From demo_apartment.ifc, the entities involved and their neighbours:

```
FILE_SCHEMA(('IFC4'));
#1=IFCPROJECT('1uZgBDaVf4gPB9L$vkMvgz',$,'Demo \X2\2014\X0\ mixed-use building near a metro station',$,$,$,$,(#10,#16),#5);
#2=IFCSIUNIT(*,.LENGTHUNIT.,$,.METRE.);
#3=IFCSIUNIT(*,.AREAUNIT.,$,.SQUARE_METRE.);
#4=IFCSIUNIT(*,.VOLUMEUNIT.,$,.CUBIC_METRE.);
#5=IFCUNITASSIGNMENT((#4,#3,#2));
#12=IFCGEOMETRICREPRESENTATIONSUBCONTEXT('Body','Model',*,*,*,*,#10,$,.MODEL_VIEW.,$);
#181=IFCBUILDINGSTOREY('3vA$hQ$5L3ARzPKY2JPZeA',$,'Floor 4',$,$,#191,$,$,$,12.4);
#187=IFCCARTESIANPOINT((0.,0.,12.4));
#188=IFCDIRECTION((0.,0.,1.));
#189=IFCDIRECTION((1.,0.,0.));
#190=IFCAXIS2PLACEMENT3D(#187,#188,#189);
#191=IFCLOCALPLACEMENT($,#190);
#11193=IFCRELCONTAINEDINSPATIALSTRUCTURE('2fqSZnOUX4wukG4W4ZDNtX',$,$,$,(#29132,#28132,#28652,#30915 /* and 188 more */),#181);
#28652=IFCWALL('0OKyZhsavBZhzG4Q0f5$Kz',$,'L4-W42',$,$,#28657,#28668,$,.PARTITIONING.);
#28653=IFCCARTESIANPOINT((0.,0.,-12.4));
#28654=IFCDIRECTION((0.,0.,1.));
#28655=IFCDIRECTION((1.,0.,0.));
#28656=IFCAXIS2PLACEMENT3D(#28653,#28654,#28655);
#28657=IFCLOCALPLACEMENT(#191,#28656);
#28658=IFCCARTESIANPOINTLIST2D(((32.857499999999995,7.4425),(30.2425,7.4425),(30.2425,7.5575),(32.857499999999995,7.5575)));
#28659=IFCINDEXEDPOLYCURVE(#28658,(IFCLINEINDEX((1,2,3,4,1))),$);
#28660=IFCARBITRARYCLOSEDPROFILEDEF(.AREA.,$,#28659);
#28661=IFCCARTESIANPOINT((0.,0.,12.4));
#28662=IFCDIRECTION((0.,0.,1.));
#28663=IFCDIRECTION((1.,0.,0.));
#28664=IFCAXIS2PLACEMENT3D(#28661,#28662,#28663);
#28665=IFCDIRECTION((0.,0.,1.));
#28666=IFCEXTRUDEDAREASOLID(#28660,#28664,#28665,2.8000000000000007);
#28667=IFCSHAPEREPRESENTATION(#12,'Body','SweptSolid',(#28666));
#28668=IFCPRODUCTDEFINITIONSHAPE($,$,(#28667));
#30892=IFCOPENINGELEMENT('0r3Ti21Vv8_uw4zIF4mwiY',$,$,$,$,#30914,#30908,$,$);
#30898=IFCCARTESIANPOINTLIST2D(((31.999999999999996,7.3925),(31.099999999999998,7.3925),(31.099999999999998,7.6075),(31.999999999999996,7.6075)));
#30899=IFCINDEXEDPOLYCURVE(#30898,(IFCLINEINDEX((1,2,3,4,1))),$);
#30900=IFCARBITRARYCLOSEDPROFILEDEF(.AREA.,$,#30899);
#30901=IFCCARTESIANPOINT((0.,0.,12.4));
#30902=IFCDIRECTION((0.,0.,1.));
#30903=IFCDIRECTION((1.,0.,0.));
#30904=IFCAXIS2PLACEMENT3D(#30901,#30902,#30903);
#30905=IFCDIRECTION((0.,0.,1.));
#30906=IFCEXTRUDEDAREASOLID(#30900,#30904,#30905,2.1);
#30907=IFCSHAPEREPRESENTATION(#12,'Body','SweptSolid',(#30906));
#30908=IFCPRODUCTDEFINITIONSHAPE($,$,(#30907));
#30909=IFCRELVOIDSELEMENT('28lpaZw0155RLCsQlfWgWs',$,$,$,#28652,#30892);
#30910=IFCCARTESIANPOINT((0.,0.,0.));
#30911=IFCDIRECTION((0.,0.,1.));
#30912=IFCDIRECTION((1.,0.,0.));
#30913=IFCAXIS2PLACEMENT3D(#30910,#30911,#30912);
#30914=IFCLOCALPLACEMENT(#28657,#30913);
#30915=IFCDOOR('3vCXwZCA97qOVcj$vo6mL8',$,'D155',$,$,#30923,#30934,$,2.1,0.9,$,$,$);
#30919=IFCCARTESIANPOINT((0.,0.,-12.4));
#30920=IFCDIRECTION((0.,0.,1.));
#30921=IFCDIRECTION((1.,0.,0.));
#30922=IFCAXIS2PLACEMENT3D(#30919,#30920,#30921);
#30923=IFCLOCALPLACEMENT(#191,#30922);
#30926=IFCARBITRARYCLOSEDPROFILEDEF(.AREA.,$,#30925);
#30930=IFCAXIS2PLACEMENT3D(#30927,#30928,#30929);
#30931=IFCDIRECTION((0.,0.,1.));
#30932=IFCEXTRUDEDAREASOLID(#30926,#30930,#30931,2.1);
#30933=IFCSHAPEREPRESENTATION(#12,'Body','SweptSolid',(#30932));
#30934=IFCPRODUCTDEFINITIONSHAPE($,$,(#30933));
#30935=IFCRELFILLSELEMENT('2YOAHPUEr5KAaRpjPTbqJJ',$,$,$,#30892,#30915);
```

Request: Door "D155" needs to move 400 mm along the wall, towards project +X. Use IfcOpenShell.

```python
import ifcopenshell
import ifcopenshell.api.geometry
import ifcopenshell.util.placement
import ifcopenshell.util.unit

model = ifcopenshell.open("demo_apartment.ifc")
unit_scale = ifcopenshell.util.unit.calculate_unit_scale(model)

door = model.by_guid("3vCXwZCA97qOVcj$vo6mL8")
opening = door.FillsVoids[0].RelatingOpeningElement
wall = opening.VoidsElements[0].RelatingBuildingElement

wall_matrix = ifcopenshell.util.placement.get_local_placement(wall.ObjectPlacement)
shift = wall_matrix[:3, 0] * 0.4 / unit_scale
before = ifcopenshell.util.placement.get_local_placement(door.ObjectPlacement)[:3, 3].copy()

# The door is not placed relative to its opening, so move both.
for product in (opening, door):
    matrix = ifcopenshell.util.placement.get_local_placement(product.ObjectPlacement)
    matrix[:3, 3] += shift
    ifcopenshell.api.geometry.edit_object_placement(model, product=product, matrix=matrix, is_si=False)

after = ifcopenshell.util.placement.get_local_placement(door.ObjectPlacement)[:3, 3]
print("door moved by", (after - before).round(3) + 0.0)

model.write("demo_apartment_updated.ifc")
```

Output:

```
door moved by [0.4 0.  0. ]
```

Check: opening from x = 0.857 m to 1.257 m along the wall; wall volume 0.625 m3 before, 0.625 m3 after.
